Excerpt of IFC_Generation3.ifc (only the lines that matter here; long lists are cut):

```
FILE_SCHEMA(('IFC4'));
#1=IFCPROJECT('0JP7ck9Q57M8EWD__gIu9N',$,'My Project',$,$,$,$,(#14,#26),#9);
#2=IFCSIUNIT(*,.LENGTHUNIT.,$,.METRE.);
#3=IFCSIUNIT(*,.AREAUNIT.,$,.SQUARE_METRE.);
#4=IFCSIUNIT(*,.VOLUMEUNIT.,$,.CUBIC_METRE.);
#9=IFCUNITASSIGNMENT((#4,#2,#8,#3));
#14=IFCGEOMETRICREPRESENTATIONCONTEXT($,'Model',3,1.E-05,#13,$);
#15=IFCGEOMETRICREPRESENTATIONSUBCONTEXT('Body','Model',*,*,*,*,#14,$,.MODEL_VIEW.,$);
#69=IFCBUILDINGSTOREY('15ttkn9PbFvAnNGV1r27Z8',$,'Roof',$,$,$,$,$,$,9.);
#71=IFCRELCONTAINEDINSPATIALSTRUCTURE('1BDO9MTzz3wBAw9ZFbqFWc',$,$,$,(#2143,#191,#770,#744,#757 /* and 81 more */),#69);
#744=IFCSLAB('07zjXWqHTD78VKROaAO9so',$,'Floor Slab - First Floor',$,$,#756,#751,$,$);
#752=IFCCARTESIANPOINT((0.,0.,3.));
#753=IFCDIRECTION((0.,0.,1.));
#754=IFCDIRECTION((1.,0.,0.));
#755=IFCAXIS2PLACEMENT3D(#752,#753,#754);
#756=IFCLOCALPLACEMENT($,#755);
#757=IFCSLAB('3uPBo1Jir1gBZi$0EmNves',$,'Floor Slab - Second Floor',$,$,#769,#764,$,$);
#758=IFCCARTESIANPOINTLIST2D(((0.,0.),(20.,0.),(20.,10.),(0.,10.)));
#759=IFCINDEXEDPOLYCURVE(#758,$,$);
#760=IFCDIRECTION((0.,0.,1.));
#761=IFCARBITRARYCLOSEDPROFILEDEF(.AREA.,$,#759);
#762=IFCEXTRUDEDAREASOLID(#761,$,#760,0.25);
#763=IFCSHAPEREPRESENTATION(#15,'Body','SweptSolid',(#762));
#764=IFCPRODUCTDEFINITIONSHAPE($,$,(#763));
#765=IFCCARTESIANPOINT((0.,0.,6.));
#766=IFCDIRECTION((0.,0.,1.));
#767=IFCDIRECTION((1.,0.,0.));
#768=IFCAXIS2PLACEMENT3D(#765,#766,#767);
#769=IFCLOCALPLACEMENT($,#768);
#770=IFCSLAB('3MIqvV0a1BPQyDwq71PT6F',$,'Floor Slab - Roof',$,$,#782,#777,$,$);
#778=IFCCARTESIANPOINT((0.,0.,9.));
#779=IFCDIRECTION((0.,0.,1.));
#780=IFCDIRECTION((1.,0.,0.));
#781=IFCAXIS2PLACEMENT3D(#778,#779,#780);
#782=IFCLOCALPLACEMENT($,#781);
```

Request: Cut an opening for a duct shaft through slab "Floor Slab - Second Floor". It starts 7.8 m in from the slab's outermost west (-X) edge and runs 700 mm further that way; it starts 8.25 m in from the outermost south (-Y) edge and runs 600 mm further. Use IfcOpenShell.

```python
import numpy as np
import ifcopenshell
import ifcopenshell.api.feature
import ifcopenshell.api.geometry
import ifcopenshell.api.root
import ifcopenshell.geom
import ifcopenshell.util.placement
import ifcopenshell.util.representation
import ifcopenshell.util.shape
import ifcopenshell.util.unit

model = ifcopenshell.open("IFC_Generation3.ifc")
unit_scale = ifcopenshell.util.unit.calculate_unit_scale(model)
settings = ifcopenshell.geom.settings()


def volume(element):
    """Net volume in cubic metres, openings subtracted."""
    shape = ifcopenshell.geom.create_shape(settings, element)
    return ifcopenshell.util.shape.get_volume(shape.geometry)


slab = model.by_guid("3uPBo1Jir1gBZi$0EmNves")
before = volume(slab)

# Extent in the slab's own axes, in metres. The edges named are its -X and -Y sides.
slab_shape = ifcopenshell.geom.create_shape(settings, slab)
vertices = ifcopenshell.util.shape.get_vertices(slab_shape.geometry)
x_min, y_min, bottom = vertices.min(axis=0)
top = vertices[:, 2].max()

opening = ifcopenshell.api.root.create_entity(model, ifc_class="IfcOpeningElement", name="Duct shaft opening", predefined_type="OPENING")
context = ifcopenshell.util.representation.get_context(model, "Model", "Body", "MODEL_VIEW")
width, depth = 0.7, 0.6
outline = [(0.0, 0.0), (width, 0.0), (width, depth), (0.0, depth), (0.0, 0.0)]
# Overshoot both faces by 50 mm so the cut is clean.
shape = ifcopenshell.api.geometry.add_slab_representation(
    model, context=context, depth=top - bottom + 0.1, polyline=outline
)
ifcopenshell.api.geometry.assign_representation(model, product=opening, representation=shape)

matrix = ifcopenshell.util.placement.get_local_placement(slab.ObjectPlacement)
matrix[:, 3] = matrix @ np.append(np.array([x_min + 7.8, y_min + 8.25, bottom - 0.05]) / unit_scale, 1.0)
ifcopenshell.api.geometry.edit_object_placement(model, product=opening, matrix=matrix, is_si=False)
ifcopenshell.api.feature.add_feature(model, feature=opening, element=slab)

after = volume(slab)

print(f"slab volume {before:.3f} -> {after:.3f} m3")

model.write("IFC_Generation3_v2.ifc")
```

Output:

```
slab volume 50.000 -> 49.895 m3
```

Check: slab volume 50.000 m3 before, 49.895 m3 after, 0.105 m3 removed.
